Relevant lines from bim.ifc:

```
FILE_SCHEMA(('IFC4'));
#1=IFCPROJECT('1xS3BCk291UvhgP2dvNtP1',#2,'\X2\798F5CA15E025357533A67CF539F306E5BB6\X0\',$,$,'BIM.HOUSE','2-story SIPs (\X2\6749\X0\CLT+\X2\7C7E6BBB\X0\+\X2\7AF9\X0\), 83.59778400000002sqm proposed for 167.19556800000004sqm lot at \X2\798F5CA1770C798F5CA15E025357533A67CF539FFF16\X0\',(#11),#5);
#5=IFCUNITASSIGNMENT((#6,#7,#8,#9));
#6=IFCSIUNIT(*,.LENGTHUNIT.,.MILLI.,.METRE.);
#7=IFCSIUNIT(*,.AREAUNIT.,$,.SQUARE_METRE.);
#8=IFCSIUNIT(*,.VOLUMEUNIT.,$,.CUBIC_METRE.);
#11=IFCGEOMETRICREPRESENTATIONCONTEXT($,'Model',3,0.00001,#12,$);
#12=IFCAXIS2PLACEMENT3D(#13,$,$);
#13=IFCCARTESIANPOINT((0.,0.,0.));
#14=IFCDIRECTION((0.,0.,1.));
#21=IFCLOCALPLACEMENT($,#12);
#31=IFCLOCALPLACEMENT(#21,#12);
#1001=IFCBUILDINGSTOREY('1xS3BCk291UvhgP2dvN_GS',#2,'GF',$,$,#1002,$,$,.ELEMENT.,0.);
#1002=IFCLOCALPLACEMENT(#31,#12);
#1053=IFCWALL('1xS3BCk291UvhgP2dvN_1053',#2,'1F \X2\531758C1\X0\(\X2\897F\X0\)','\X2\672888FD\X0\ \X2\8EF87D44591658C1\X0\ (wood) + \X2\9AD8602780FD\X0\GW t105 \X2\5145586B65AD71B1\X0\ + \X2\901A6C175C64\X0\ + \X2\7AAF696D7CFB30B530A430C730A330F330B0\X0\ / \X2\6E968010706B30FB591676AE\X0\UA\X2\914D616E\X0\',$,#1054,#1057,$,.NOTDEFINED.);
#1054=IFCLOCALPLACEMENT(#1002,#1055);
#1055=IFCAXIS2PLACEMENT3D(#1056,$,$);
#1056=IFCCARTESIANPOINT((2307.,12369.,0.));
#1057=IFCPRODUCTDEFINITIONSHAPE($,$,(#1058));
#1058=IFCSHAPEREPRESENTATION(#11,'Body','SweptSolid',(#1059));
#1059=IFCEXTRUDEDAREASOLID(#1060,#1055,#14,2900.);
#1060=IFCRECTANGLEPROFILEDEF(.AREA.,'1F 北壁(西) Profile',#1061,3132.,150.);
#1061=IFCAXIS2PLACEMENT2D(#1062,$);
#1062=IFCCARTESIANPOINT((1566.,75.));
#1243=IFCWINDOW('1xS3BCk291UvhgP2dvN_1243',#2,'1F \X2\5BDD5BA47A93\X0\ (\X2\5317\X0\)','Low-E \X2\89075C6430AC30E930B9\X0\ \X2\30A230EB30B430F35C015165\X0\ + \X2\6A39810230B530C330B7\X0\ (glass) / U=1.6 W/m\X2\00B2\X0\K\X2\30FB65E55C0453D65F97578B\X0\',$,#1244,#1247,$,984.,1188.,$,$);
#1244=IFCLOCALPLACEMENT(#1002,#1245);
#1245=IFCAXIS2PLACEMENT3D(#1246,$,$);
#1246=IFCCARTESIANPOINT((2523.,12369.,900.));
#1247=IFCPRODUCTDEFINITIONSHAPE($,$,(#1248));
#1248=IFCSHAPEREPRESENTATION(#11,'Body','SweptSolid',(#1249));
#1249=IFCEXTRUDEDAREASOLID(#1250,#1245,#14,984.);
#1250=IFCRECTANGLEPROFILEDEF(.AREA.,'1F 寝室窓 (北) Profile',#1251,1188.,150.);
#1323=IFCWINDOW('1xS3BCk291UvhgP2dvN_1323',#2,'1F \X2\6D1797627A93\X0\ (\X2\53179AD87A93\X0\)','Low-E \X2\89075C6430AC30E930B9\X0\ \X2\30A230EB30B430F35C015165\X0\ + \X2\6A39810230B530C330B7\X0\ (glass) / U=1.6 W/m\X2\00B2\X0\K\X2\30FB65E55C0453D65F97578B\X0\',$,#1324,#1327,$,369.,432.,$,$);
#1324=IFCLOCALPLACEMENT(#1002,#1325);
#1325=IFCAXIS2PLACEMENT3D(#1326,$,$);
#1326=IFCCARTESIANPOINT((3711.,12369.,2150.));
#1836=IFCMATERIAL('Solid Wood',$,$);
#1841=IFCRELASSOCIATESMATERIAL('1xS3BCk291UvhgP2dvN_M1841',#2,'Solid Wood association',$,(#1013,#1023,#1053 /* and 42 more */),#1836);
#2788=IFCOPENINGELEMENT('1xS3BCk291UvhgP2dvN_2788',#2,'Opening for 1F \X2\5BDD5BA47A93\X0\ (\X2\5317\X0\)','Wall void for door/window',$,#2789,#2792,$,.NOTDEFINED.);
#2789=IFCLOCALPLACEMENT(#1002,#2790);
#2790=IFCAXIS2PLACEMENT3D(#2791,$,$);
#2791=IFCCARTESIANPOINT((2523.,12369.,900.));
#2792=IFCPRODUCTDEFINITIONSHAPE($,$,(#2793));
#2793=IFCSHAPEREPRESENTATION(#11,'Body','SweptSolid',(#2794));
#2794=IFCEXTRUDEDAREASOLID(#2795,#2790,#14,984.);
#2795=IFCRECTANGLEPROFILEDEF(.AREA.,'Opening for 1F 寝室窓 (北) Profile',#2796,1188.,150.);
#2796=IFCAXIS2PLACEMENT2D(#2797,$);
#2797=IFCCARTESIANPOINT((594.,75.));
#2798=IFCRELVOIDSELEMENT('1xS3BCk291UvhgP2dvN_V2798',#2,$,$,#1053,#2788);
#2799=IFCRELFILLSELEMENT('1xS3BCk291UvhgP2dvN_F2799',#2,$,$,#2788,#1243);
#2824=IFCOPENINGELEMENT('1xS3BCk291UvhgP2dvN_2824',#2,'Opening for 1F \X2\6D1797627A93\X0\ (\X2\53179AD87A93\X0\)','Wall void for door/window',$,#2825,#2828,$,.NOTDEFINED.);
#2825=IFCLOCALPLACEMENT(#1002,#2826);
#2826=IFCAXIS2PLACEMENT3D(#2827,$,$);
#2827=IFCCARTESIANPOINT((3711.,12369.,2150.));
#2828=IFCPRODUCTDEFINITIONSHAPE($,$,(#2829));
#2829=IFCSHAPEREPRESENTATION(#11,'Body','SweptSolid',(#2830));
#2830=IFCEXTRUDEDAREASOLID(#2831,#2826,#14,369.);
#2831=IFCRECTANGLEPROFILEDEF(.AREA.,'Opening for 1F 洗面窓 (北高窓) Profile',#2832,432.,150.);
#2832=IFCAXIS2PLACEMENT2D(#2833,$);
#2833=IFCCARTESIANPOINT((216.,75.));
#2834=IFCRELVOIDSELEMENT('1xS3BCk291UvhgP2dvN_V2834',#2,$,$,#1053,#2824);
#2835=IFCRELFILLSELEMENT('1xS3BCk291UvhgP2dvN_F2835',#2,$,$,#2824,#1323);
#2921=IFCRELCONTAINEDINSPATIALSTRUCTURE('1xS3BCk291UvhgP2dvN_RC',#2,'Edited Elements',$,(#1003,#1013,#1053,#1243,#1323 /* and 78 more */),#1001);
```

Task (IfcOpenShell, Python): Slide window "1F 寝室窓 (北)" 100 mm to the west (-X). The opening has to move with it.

```python
import ifcopenshell
import ifcopenshell.api.geometry
import ifcopenshell.util.placement

model = ifcopenshell.open("bim.ifc")

window = model.by_id(1243)
opening = window.FillsVoids[0].RelatingOpeningElement
wall = opening.VoidsElements[0].RelatingBuildingElement

wall_matrix = ifcopenshell.util.placement.get_local_placement(wall.ObjectPlacement)
shift = wall_matrix[:3, 0] * -100.0
before = ifcopenshell.util.placement.get_local_placement(window.ObjectPlacement)[:3, 3].copy()

# The window is not placed relative to its opening, so move both.
for product in (opening, window):
    matrix = ifcopenshell.util.placement.get_local_placement(product.ObjectPlacement)
    matrix[:3, 3] += shift
    ifcopenshell.api.geometry.edit_object_placement(model, product=product, matrix=matrix, is_si=False)

after = ifcopenshell.util.placement.get_local_placement(window.ObjectPlacement)[:3, 3]
print("window moved by", (after - before).round(3) + 0.0)

model.write("bim_updated.ifc")
```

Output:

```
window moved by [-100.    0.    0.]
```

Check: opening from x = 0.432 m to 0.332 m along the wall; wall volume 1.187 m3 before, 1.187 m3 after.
